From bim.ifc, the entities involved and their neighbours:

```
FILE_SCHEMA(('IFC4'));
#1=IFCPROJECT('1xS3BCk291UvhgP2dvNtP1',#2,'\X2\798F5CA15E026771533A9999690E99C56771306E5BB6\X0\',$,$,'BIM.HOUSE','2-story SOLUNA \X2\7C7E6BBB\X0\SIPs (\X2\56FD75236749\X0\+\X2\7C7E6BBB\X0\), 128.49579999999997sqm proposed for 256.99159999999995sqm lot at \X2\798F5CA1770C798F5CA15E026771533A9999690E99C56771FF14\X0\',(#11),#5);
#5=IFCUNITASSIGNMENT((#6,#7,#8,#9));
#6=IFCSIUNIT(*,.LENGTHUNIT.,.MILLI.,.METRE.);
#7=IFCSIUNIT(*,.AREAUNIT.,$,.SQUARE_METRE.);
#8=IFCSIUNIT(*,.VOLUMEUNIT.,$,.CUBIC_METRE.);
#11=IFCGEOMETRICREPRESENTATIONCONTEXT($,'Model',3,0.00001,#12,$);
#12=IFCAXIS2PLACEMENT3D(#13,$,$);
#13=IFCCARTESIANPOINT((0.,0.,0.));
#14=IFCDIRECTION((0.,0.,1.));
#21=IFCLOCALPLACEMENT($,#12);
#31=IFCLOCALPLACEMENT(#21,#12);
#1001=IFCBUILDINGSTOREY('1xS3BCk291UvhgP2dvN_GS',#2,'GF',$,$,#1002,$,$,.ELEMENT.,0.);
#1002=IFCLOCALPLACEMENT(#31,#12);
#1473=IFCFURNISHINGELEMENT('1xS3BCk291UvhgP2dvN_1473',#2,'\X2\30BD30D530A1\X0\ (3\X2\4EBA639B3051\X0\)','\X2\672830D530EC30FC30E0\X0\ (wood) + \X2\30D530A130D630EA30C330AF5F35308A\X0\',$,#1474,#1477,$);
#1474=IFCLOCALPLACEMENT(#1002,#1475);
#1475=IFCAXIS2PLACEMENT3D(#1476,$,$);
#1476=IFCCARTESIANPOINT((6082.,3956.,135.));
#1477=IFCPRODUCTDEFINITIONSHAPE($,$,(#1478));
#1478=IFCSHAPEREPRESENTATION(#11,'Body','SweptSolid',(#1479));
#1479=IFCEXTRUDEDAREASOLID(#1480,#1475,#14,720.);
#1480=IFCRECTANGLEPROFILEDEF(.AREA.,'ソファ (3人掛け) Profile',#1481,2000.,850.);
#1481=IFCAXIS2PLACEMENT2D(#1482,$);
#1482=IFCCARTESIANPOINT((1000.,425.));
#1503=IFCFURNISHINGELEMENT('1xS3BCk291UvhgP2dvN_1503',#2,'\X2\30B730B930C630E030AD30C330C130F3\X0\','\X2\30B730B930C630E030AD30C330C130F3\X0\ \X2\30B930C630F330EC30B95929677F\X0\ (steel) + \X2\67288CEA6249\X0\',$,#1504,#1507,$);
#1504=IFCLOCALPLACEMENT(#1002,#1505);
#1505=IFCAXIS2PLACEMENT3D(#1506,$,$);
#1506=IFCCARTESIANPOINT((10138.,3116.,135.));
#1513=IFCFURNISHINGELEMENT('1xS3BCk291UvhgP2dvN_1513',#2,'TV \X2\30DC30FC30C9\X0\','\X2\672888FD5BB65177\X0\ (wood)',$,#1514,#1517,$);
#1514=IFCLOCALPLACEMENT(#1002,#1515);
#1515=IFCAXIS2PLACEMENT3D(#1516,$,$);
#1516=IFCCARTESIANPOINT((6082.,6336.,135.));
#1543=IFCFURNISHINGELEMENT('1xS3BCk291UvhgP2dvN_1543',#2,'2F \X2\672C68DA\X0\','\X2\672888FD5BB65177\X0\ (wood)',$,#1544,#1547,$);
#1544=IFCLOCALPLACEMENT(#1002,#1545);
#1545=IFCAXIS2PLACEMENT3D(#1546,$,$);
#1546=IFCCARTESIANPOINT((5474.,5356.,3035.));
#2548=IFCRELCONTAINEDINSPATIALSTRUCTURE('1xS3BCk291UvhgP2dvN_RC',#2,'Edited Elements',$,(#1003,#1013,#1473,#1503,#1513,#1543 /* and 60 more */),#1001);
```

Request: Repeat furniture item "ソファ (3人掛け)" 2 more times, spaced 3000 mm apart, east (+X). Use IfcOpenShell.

```python
import numpy as np
import ifcopenshell
import ifcopenshell.api.geometry
import ifcopenshell.api.root
import ifcopenshell.util.element
import ifcopenshell.util.placement
import ifcopenshell.util.unit

model = ifcopenshell.open("bim.ifc")
unit_scale = ifcopenshell.util.unit.calculate_unit_scale(model)


def reuse_history(source, copy):
    """copy_class also copies each property set's owner history, people and application; keep the originals."""
    for rel in copy.IsDefinedBy:
        if rel.is_a("IfcRelDefinesByProperties") and (history := rel.RelatingPropertyDefinition.OwnerHistory):
            rel.RelatingPropertyDefinition.OwnerHistory = source.OwnerHistory
            ifcopenshell.util.element.remove_deep2(model, history)


source = model.by_guid("1xS3BCk291UvhgP2dvN_1473")
base = ifcopenshell.util.placement.get_local_placement(source.ObjectPlacement)
step = np.array([1.0, 0.0, 0.0]) * 3 / unit_scale

for i in range(1, 3):
    copy = ifcopenshell.api.root.copy_class(model, product=source)
    copy.Representation = ifcopenshell.util.element.copy_deep(
        model, source.Representation, exclude=["IfcGeometricRepresentationContext", "IfcRepresentationMap"]
    )
    reuse_history(source, copy)
    matrix = base.copy()
    matrix[:3, 3] += i * step
    print("added at", matrix[:3, 3].round(3) + 0.0)
    ifcopenshell.api.geometry.edit_object_placement(model, product=copy, matrix=matrix, is_si=False)

model.write("bim_updated.ifc")
```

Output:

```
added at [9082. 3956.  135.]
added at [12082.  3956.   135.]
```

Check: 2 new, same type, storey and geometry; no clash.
